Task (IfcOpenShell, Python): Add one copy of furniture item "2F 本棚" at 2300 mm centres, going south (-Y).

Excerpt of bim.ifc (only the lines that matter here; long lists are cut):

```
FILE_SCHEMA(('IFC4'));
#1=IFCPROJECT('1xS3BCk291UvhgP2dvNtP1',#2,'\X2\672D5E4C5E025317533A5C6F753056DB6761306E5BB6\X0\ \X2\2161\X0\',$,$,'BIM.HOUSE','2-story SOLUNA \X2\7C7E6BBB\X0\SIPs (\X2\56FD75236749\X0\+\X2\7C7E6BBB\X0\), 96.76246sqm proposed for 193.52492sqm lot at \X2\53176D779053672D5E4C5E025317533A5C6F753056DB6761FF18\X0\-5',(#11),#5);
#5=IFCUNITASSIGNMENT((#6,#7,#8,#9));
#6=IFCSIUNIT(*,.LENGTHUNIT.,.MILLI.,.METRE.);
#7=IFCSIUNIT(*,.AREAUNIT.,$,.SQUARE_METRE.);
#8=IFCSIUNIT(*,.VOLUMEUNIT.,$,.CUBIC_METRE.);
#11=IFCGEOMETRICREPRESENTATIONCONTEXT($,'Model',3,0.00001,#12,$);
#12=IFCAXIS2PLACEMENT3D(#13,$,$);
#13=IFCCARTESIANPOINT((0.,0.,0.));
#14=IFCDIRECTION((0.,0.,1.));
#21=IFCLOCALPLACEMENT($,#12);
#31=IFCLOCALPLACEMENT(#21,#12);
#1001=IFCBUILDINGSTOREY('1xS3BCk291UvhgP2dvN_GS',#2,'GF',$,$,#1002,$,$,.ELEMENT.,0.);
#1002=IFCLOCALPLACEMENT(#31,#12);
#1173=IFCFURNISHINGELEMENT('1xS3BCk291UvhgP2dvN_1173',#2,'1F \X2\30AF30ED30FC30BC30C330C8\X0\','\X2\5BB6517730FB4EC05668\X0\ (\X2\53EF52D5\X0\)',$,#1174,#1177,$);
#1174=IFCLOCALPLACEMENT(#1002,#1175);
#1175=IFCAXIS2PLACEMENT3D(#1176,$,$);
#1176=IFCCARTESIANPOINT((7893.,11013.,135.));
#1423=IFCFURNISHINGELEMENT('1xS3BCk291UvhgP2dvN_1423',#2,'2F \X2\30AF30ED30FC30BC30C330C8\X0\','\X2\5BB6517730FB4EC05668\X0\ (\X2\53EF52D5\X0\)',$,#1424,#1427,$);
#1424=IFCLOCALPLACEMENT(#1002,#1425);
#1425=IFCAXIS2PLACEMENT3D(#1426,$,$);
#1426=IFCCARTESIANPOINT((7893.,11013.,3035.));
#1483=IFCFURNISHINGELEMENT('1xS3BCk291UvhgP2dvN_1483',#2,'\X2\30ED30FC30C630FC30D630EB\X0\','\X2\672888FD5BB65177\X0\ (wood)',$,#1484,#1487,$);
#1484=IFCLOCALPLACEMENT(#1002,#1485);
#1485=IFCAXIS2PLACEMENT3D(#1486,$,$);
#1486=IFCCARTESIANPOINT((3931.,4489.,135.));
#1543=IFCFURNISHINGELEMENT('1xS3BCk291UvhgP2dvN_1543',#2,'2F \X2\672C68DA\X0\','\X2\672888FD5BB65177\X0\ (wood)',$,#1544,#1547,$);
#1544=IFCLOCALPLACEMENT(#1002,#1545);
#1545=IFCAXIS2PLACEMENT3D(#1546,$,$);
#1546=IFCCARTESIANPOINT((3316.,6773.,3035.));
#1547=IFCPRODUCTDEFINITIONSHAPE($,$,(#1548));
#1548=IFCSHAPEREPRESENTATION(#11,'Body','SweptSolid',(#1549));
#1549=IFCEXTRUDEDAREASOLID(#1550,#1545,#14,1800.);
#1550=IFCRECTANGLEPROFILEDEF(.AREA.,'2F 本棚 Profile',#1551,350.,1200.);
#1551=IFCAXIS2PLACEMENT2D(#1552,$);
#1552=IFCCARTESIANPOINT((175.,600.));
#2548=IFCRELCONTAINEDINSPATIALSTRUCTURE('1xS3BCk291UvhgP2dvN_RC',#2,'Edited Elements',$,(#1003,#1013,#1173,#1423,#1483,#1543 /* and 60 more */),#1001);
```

```python
import numpy as np
import ifcopenshell
import ifcopenshell.api.geometry
import ifcopenshell.api.root
import ifcopenshell.util.element
import ifcopenshell.util.placement
import ifcopenshell.util.unit

model = ifcopenshell.open("bim.ifc")
unit_scale = ifcopenshell.util.unit.calculate_unit_scale(model)


def reuse_history(source, copy):
    """copy_class also copies each property set's owner history, people and application; keep the originals."""
    for rel in copy.IsDefinedBy:
        if rel.is_a("IfcRelDefinesByProperties") and (history := rel.RelatingPropertyDefinition.OwnerHistory):
            rel.RelatingPropertyDefinition.OwnerHistory = source.OwnerHistory
            ifcopenshell.util.element.remove_deep2(model, history)


source = model.by_id(1543)
base = ifcopenshell.util.placement.get_local_placement(source.ObjectPlacement)
step = np.array([0.0, -1.0, 0.0]) * 2.3 / unit_scale

for i in range(1, 2):
    copy = ifcopenshell.api.root.copy_class(model, product=source)
    copy.Representation = ifcopenshell.util.element.copy_deep(
        model, source.Representation, exclude=["IfcGeometricRepresentationContext", "IfcRepresentationMap"]
    )
    reuse_history(source, copy)
    matrix = base.copy()
    matrix[:3, 3] += i * step
    print("added at", matrix[:3, 3].round(3) + 0.0)
    ifcopenshell.api.geometry.edit_object_placement(model, product=copy, matrix=matrix, is_si=False)

model.write("bim-out.ifc")
```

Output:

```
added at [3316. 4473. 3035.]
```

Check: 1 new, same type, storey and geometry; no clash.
